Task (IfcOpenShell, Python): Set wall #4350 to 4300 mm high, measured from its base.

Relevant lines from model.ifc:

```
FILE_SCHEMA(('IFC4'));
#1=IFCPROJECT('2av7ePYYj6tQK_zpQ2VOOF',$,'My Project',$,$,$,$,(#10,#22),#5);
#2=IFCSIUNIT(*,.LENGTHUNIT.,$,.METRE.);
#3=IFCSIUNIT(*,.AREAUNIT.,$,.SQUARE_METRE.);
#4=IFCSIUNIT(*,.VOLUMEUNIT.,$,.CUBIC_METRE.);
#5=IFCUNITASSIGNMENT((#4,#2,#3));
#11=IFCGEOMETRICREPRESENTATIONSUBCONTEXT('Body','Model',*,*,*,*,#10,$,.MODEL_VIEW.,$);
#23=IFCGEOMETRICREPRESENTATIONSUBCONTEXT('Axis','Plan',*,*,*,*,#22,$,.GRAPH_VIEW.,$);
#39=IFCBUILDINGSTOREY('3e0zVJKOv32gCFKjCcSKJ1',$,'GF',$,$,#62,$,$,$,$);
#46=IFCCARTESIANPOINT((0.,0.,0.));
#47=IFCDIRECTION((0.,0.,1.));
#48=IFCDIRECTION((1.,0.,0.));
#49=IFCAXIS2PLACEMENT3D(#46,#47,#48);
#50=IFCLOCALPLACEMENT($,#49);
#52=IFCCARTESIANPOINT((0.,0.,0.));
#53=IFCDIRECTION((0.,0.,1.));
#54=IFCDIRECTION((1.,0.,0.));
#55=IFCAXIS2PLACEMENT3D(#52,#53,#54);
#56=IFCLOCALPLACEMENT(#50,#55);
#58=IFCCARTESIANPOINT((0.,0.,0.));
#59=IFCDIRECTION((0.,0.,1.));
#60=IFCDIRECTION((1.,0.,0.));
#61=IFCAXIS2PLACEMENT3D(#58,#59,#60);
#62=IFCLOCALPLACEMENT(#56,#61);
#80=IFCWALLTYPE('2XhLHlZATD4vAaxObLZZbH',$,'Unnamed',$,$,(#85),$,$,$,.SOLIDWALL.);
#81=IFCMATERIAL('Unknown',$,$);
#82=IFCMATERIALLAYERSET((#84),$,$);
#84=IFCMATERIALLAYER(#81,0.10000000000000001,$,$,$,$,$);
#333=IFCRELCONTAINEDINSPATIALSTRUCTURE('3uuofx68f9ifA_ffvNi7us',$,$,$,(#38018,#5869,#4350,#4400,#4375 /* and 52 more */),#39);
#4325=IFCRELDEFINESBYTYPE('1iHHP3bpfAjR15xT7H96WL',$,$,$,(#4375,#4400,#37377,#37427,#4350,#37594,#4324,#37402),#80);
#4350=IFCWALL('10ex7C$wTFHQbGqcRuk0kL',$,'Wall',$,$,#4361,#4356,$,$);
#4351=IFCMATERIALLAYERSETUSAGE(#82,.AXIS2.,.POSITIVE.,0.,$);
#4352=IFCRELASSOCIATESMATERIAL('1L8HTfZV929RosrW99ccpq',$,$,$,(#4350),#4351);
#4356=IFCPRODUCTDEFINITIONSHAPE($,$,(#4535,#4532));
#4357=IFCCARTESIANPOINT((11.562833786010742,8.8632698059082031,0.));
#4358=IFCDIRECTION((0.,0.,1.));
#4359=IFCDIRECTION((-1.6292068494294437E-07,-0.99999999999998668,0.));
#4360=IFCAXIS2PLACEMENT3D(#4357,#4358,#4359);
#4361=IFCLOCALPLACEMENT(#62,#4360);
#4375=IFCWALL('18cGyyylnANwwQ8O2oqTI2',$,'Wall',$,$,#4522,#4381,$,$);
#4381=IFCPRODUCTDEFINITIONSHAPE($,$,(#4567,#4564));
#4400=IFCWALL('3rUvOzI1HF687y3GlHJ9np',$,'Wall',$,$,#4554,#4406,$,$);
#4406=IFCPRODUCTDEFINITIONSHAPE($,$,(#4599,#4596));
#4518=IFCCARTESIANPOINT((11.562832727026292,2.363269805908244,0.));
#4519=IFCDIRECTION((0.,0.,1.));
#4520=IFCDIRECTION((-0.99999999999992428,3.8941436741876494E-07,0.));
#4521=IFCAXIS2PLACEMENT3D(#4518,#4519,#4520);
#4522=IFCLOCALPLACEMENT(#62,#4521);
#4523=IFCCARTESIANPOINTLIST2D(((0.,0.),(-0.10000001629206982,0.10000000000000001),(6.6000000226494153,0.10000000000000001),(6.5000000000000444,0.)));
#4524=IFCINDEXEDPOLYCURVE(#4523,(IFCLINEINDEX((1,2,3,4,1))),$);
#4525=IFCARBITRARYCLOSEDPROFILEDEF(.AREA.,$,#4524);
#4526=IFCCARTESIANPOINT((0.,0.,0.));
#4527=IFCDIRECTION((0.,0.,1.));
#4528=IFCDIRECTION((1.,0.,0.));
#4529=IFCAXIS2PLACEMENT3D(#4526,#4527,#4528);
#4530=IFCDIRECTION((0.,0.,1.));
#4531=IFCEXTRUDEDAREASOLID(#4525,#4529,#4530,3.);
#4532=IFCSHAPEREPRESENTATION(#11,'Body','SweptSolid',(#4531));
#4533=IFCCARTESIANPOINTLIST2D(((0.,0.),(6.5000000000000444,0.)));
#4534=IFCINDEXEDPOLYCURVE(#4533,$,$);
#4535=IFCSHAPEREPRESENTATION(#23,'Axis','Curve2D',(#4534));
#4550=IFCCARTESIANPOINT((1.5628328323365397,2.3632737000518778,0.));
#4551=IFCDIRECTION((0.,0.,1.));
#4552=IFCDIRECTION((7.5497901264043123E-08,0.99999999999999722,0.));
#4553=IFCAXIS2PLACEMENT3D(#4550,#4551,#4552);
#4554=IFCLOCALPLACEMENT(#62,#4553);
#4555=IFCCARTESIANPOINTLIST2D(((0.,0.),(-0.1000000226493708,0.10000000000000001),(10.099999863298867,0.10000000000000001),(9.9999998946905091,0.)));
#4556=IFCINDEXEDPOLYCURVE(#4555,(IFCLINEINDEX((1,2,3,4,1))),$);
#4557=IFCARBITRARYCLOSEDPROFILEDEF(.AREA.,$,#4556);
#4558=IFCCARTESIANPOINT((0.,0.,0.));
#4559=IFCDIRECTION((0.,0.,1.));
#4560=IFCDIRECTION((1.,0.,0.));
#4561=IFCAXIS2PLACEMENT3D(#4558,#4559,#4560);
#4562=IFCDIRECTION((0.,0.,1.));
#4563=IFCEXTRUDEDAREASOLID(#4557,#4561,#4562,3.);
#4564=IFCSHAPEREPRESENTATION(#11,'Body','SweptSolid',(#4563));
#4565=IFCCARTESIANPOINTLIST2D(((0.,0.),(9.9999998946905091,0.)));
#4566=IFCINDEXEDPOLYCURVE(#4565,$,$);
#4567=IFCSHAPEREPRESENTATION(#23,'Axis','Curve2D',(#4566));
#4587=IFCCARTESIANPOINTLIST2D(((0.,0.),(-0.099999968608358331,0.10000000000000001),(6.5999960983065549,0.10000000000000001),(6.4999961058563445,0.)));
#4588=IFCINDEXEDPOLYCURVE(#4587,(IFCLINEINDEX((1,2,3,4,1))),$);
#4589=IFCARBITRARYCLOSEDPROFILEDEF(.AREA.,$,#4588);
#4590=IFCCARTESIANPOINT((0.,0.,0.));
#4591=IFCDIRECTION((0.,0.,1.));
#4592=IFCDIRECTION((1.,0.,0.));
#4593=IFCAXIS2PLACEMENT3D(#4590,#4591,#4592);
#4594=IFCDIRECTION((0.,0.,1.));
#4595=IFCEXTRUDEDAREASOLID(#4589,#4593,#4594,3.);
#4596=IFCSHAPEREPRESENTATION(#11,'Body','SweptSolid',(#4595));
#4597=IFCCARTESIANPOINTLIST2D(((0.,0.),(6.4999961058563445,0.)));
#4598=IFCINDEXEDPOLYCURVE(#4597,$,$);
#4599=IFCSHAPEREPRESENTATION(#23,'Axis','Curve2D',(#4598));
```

```python
import ifcopenshell
import ifcopenshell.geom
import ifcopenshell.util.representation
import ifcopenshell.util.shape

model = ifcopenshell.open("model.ifc")
settings = ifcopenshell.geom.settings()


def volume(element):
    """Net volume in cubic metres, openings subtracted."""
    shape = ifcopenshell.geom.create_shape(settings, element)
    return ifcopenshell.util.shape.get_volume(shape.geometry)


wall = model.by_guid("10ex7C$wTFHQbGqcRuk0kL")
before = volume(wall)

body = ifcopenshell.util.representation.get_representation(wall, "Model", "Body")
solid = body.Items[0]
old_height = solid.Depth
solid.Depth = 4.3
after = volume(wall)

print(f"height {old_height:g} -> {solid.Depth:g}, volume {before:.3f} -> {after:.3f} m3")

model.write("model_updated.ifc")
```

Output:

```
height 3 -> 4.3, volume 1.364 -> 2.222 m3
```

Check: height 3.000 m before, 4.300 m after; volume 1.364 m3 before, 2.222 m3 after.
